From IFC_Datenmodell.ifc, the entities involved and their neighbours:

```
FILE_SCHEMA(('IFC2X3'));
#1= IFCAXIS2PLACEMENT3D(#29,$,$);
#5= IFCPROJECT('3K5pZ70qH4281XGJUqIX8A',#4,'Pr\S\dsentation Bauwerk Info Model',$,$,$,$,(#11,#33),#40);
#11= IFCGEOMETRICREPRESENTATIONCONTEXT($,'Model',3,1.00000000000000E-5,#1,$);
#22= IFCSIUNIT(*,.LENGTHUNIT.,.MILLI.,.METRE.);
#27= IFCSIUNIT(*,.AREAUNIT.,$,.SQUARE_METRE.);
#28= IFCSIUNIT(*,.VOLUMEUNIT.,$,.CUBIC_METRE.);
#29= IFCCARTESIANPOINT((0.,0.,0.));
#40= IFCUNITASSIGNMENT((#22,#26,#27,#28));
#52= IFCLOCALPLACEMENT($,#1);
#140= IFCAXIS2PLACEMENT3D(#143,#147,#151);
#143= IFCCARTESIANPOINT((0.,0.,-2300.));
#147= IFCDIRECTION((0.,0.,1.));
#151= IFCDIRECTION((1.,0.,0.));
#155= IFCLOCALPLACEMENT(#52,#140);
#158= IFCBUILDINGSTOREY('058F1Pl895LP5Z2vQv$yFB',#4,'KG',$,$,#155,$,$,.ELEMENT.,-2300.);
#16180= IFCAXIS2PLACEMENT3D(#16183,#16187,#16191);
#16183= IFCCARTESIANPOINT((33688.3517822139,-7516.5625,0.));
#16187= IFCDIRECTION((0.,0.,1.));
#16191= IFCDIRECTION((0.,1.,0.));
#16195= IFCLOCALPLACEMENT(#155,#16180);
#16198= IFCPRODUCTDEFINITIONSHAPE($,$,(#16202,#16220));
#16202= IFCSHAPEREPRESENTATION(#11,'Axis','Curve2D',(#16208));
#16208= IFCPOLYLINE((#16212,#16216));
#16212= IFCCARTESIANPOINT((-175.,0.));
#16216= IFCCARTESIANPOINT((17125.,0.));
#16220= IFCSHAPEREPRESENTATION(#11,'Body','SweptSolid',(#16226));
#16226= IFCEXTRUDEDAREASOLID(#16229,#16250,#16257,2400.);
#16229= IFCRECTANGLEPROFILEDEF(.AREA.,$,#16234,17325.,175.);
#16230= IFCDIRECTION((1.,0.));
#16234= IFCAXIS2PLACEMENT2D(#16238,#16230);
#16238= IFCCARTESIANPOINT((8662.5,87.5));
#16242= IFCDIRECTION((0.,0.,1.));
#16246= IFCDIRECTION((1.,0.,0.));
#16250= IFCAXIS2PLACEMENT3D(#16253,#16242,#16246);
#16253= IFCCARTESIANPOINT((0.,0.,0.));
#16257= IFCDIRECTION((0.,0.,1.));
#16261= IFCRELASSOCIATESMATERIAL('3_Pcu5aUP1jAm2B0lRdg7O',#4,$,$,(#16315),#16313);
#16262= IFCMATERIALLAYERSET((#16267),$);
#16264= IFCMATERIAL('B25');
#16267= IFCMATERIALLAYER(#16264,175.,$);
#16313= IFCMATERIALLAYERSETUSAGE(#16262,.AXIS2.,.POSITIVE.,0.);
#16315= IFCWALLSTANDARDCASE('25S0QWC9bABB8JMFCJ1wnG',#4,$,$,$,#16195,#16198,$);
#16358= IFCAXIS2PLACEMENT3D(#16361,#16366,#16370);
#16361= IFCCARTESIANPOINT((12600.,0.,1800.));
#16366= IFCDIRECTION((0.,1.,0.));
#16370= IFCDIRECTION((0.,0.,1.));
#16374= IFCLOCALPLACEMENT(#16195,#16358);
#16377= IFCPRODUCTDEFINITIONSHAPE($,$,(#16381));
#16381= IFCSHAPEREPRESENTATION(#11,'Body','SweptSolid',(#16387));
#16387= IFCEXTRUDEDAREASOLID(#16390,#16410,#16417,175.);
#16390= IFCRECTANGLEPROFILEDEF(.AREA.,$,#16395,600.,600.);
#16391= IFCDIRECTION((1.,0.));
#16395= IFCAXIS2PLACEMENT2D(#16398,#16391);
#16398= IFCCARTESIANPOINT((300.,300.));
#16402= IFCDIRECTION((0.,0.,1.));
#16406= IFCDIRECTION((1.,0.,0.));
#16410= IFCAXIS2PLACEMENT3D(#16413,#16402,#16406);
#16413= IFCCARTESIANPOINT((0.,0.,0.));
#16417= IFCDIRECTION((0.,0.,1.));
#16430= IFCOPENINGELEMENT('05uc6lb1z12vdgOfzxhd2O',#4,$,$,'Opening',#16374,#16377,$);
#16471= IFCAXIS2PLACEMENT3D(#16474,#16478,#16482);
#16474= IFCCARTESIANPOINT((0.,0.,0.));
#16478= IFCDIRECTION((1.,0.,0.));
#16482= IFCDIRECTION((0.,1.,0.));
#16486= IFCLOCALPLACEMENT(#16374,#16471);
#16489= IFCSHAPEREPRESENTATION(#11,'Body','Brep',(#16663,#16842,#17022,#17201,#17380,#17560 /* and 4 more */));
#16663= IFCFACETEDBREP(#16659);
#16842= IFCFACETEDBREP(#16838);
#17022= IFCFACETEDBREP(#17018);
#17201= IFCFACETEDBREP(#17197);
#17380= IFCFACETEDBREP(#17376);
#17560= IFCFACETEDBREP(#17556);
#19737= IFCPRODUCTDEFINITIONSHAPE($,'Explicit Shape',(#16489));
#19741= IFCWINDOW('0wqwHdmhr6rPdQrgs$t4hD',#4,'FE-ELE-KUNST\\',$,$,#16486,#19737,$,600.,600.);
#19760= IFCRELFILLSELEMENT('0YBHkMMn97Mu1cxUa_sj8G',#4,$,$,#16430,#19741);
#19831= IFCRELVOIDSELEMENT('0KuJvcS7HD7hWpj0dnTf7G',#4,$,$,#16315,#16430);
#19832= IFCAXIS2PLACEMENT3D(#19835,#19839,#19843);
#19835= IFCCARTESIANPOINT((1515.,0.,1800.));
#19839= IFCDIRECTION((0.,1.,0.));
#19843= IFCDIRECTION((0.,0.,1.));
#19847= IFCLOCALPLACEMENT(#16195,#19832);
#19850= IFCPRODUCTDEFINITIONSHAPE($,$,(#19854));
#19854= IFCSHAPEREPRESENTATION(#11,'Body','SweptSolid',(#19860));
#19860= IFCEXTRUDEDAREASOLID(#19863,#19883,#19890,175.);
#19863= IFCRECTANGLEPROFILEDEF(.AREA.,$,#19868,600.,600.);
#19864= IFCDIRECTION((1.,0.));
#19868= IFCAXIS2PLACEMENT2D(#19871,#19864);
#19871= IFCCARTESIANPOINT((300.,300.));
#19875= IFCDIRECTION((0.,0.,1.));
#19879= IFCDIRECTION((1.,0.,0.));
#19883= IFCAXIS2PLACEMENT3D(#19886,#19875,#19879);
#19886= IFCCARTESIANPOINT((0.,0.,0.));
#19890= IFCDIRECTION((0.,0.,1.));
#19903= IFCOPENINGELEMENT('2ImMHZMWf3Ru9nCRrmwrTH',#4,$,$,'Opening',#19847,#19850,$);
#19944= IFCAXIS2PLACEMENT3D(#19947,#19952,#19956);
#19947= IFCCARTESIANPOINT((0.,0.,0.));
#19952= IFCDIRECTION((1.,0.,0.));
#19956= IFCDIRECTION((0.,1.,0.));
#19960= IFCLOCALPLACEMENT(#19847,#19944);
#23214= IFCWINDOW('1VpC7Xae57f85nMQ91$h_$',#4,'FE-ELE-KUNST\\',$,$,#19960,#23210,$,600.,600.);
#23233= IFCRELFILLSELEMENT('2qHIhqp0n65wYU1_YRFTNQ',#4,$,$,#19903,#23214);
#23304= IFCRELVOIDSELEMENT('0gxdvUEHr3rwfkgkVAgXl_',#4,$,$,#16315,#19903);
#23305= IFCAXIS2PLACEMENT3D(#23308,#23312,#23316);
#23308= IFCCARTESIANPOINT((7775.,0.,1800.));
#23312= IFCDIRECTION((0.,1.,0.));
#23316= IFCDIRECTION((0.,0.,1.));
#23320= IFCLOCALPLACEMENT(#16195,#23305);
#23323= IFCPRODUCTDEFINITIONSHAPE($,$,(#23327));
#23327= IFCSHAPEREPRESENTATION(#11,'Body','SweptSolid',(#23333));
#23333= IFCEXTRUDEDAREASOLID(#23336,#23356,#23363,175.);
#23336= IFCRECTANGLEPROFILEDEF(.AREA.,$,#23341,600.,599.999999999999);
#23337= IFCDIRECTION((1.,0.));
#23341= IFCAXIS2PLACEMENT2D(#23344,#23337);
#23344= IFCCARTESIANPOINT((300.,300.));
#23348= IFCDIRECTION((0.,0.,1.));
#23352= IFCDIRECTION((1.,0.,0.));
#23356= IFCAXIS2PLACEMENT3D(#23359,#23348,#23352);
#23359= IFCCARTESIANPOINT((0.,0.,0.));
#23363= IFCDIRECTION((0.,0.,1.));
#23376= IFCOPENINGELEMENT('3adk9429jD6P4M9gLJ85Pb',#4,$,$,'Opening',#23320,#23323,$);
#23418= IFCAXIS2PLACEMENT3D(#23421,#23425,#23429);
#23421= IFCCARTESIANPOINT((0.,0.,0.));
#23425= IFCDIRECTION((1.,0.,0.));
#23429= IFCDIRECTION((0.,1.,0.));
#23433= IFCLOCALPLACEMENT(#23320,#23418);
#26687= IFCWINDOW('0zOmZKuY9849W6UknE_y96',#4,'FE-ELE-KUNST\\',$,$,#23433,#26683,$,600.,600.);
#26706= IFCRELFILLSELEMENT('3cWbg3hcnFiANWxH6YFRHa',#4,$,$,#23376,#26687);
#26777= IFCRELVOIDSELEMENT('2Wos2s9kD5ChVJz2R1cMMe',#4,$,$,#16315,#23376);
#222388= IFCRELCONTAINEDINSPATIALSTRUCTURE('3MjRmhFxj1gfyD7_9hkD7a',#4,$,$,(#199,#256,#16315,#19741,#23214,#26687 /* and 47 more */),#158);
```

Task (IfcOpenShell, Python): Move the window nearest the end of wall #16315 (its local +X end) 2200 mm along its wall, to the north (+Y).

```python
import ifcopenshell
import ifcopenshell.api.geometry
import ifcopenshell.util.placement

model = ifcopenshell.open("IFC_Datenmodell.ifc")

window = model.by_guid("0wqwHdmhr6rPdQrgs$t4hD")
opening = window.FillsVoids[0].RelatingOpeningElement
wall = opening.VoidsElements[0].RelatingBuildingElement

wall_matrix = ifcopenshell.util.placement.get_local_placement(wall.ObjectPlacement)
shift = wall_matrix[:3, 0] * 2200.0
before = ifcopenshell.util.placement.get_local_placement(window.ObjectPlacement)[:3, 3].copy()

# The window is placed relative to its opening, so it follows when the opening moves.
matrix = ifcopenshell.util.placement.get_local_placement(opening.ObjectPlacement)
matrix[:3, 3] += shift
ifcopenshell.api.geometry.edit_object_placement(
    model, product=opening, matrix=matrix, is_si=False, should_transform_children=True
)

after = ifcopenshell.util.placement.get_local_placement(window.ObjectPlacement)[:3, 3]
print("window moved by", (after - before).round(3) + 0.0)

model.write("IFC_Datenmodell-out.ifc")
```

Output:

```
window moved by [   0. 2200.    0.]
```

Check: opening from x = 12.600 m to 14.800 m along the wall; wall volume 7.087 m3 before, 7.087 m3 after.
